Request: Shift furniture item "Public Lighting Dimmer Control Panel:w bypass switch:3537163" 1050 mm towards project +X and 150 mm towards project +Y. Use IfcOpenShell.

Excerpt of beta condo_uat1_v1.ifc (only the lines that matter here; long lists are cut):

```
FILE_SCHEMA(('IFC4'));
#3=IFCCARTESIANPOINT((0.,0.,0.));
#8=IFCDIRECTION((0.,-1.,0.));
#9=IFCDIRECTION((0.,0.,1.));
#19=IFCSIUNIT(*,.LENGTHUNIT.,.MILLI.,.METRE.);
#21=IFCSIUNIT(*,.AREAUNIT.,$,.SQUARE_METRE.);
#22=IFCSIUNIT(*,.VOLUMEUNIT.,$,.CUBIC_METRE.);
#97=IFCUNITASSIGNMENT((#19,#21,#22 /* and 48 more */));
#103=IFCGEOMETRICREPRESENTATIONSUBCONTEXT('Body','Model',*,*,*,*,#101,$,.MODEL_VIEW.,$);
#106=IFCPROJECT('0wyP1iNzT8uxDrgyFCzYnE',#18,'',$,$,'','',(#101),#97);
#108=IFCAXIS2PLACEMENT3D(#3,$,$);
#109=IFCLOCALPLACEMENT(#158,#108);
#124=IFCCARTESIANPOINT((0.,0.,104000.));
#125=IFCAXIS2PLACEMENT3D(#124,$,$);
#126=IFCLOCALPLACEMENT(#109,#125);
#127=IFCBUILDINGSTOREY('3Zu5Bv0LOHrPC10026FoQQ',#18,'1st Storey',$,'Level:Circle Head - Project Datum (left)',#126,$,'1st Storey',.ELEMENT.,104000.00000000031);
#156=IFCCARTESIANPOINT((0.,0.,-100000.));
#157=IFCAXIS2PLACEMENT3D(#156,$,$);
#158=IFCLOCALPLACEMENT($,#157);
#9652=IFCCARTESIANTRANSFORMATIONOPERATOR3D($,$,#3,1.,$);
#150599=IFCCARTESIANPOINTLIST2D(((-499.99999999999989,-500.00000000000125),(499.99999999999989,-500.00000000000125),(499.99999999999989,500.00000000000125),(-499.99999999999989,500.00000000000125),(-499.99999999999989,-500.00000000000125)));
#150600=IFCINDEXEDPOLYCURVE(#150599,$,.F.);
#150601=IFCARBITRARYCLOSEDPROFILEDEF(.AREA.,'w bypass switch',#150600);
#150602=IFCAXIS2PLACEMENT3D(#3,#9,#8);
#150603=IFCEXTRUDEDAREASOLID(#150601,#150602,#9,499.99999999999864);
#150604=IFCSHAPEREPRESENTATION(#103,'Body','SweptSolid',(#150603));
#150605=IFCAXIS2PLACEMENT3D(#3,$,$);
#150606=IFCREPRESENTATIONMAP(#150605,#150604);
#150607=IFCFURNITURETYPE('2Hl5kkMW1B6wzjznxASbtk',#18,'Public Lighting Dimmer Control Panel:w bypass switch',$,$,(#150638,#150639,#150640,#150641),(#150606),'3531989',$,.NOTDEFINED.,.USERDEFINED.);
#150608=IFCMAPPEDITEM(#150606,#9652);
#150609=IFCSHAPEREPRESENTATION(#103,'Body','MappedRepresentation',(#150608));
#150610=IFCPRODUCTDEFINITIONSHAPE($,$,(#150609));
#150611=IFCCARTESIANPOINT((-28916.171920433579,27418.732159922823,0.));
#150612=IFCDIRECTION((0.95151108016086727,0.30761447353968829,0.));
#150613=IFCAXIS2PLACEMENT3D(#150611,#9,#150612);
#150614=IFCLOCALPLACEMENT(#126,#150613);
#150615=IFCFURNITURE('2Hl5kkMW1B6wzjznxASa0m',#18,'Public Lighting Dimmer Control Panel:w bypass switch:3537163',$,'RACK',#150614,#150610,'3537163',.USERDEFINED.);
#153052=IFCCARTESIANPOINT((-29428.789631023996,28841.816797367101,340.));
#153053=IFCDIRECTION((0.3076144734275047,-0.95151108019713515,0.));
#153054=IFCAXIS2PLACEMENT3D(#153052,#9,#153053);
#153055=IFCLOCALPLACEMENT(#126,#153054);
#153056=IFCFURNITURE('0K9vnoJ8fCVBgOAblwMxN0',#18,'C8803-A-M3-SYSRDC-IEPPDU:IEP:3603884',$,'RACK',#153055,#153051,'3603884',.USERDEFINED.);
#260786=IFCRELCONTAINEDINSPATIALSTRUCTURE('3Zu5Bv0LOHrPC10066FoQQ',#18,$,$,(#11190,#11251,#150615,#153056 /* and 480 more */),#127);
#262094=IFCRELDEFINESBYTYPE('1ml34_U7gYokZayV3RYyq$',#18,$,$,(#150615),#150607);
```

```python
import ifcopenshell
import ifcopenshell.api.geometry
import ifcopenshell.util.placement

model = ifcopenshell.open("beta condo_uat1_v1.ifc")

item = model.by_guid("2Hl5kkMW1B6wzjznxASa0m")
matrix = ifcopenshell.util.placement.get_local_placement(item.ObjectPlacement)
matrix[0, 3] += 1050.0
matrix[1, 3] += 150.0
ifcopenshell.api.geometry.edit_object_placement(model, product=item, matrix=matrix, is_si=False)

print(ifcopenshell.util.placement.get_local_placement(item.ObjectPlacement).round(3) + 0.0)

model.write("beta condo_uat1_v1-out.ifc")
```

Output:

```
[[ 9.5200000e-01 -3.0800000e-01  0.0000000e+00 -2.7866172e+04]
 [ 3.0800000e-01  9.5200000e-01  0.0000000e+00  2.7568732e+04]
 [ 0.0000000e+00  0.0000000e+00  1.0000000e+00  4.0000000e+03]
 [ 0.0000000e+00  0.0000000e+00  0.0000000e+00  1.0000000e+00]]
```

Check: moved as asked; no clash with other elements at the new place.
